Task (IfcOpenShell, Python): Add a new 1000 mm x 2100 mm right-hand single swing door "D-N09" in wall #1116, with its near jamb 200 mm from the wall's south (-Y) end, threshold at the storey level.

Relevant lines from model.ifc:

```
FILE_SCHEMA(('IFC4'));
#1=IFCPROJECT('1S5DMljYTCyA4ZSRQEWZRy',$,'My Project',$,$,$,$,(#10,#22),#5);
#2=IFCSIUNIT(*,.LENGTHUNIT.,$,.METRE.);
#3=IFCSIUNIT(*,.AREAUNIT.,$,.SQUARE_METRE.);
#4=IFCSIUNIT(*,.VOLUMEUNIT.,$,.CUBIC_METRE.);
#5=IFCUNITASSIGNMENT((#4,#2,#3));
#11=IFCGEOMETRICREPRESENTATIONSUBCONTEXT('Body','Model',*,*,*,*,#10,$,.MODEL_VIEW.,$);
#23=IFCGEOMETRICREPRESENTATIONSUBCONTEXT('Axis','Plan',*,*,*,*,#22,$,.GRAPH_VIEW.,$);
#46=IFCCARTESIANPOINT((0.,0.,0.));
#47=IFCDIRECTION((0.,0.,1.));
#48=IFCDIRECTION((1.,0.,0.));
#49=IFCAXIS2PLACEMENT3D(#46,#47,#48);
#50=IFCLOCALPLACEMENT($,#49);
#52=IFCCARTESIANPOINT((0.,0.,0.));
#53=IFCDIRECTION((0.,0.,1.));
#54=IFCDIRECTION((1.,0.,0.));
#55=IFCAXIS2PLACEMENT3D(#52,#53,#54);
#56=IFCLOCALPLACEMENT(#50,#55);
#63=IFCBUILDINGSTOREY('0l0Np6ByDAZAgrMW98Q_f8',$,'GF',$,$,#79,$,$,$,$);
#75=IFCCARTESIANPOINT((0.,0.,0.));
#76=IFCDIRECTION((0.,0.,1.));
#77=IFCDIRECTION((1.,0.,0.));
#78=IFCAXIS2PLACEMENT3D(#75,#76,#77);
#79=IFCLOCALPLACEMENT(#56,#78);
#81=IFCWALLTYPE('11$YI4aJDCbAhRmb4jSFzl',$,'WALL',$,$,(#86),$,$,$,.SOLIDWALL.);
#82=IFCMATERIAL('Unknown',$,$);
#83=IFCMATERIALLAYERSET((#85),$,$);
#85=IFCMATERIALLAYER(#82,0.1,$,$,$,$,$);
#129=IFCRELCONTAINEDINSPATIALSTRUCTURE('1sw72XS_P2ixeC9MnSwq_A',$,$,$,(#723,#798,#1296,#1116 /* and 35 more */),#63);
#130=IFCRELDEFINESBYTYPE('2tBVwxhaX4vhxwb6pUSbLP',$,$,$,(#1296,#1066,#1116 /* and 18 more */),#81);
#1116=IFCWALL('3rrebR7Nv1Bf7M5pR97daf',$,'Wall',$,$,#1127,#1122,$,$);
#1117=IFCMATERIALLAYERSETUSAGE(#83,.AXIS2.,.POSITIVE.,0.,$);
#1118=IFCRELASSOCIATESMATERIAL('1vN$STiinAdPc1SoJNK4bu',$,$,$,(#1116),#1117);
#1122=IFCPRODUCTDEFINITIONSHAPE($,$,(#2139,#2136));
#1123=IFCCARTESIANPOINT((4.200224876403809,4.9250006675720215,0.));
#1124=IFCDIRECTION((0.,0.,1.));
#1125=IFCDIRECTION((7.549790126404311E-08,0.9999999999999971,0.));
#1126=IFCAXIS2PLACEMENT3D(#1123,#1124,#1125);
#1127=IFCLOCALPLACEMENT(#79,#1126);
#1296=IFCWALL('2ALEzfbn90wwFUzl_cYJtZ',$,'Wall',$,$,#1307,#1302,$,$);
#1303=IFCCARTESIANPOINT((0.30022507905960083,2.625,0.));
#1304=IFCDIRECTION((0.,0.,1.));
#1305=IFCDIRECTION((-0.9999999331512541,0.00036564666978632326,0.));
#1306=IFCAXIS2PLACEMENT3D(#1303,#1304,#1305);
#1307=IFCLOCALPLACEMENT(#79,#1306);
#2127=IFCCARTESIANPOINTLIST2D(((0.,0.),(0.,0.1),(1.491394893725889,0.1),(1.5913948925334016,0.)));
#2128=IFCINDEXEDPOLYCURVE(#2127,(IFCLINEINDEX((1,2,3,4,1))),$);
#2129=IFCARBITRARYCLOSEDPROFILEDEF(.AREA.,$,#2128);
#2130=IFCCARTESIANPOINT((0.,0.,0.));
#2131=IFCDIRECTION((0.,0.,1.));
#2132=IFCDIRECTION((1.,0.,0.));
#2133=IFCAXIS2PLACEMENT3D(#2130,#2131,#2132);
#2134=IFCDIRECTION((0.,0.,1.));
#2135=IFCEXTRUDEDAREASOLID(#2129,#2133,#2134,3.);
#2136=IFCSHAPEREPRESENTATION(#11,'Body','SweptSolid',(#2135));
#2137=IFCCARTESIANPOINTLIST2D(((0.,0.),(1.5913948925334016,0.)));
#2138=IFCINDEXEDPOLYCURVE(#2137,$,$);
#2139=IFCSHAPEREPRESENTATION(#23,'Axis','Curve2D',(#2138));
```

```python
import numpy as np
import ifcopenshell
import ifcopenshell.api.feature
import ifcopenshell.api.geometry
import ifcopenshell.api.root
import ifcopenshell.api.spatial
import ifcopenshell.geom
import ifcopenshell.util.element
import ifcopenshell.util.placement
import ifcopenshell.util.representation
import ifcopenshell.util.shape
import ifcopenshell.util.unit

model = ifcopenshell.open("model.ifc")
unit_scale = ifcopenshell.util.unit.calculate_unit_scale(model)
settings = ifcopenshell.geom.settings()


def volume(element):
    """Net volume in cubic metres, openings subtracted."""
    shape = ifcopenshell.geom.create_shape(settings, element)
    return ifcopenshell.util.shape.get_volume(shape.geometry)


wall = model.by_guid("3rrebR7Nv1Bf7M5pR97daf")
storey = ifcopenshell.util.element.get_container(wall, ifc_class="IfcBuildingStorey")
context = ifcopenshell.util.representation.get_context(model, "Model", "Body", "MODEL_VIEW")
before = volume(wall)

width, height, from_end, sill = 1, 2.1, 0.2, 0.0  # metres

# The wall runs along its own X axis, and the end named is its -X end.
wall_shape = ifcopenshell.geom.create_shape(settings, wall)
x, y, z = ifcopenshell.util.shape.get_vertices(wall_shape.geometry).T
start = x.min() + from_end
face, thickness = float(y.min()), float(y.max() - y.min())
wall_matrix = ifcopenshell.util.placement.get_local_placement(wall.ObjectPlacement)
level = ifcopenshell.util.placement.get_local_placement(storey.ObjectPlacement)[2, 3]


def in_wall(x, y):
    """Placement at x, y metres in the wall's axes, at sill height."""
    matrix = wall_matrix.copy()
    matrix[:, 3] = wall_matrix @ np.array([x / unit_scale, y / unit_scale, 0.0, 1.0])
    matrix[2, 3] = level + sill / unit_scale
    return matrix


# Opening: a box that overshoots both wall faces by 50 mm.
opening = ifcopenshell.api.root.create_entity(model, ifc_class="IfcOpeningElement", predefined_type="OPENING")
box = ifcopenshell.api.geometry.add_wall_representation(
    model, context=context, length=width, height=height, thickness=thickness + 0.1
)
ifcopenshell.api.geometry.assign_representation(model, product=opening, representation=box)
ifcopenshell.api.geometry.edit_object_placement(model, product=opening, matrix=in_wall(start, face - 0.05), is_si=False)
ifcopenshell.api.feature.add_feature(model, feature=opening, element=wall)

door = ifcopenshell.api.root.create_entity(model, ifc_class="IfcDoor", name="D-N09", predefined_type="DOOR")
door.OverallWidth, door.OverallHeight = width / unit_scale, height / unit_scale
door.OperationType = "SINGLE_SWING_RIGHT"
body = ifcopenshell.api.geometry.add_door_representation(
    model,
    context=context,
    overall_width=door.OverallWidth,
    overall_height=door.OverallHeight,
    operation_type="SINGLE_SWING_RIGHT",
    lining_properties={"LiningDepth": thickness / unit_scale, "ThresholdDepth": thickness / unit_scale},
)
ifcopenshell.api.geometry.assign_representation(model, product=door, representation=body)
ifcopenshell.api.spatial.assign_container(model, products=[door], relating_structure=storey)
ifcopenshell.api.feature.add_filling(model, opening=opening, element=door)

# The lining spans the wall, so the door starts at the wall face.
ifcopenshell.api.geometry.edit_object_placement(model, product=door, matrix=in_wall(start, face), is_si=False)

after = volume(wall)

print(f"wall volume {before:.3f} -> {after:.3f} m3")

model.write("model_v2.ifc")
```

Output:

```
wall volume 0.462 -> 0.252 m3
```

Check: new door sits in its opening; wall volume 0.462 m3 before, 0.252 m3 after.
